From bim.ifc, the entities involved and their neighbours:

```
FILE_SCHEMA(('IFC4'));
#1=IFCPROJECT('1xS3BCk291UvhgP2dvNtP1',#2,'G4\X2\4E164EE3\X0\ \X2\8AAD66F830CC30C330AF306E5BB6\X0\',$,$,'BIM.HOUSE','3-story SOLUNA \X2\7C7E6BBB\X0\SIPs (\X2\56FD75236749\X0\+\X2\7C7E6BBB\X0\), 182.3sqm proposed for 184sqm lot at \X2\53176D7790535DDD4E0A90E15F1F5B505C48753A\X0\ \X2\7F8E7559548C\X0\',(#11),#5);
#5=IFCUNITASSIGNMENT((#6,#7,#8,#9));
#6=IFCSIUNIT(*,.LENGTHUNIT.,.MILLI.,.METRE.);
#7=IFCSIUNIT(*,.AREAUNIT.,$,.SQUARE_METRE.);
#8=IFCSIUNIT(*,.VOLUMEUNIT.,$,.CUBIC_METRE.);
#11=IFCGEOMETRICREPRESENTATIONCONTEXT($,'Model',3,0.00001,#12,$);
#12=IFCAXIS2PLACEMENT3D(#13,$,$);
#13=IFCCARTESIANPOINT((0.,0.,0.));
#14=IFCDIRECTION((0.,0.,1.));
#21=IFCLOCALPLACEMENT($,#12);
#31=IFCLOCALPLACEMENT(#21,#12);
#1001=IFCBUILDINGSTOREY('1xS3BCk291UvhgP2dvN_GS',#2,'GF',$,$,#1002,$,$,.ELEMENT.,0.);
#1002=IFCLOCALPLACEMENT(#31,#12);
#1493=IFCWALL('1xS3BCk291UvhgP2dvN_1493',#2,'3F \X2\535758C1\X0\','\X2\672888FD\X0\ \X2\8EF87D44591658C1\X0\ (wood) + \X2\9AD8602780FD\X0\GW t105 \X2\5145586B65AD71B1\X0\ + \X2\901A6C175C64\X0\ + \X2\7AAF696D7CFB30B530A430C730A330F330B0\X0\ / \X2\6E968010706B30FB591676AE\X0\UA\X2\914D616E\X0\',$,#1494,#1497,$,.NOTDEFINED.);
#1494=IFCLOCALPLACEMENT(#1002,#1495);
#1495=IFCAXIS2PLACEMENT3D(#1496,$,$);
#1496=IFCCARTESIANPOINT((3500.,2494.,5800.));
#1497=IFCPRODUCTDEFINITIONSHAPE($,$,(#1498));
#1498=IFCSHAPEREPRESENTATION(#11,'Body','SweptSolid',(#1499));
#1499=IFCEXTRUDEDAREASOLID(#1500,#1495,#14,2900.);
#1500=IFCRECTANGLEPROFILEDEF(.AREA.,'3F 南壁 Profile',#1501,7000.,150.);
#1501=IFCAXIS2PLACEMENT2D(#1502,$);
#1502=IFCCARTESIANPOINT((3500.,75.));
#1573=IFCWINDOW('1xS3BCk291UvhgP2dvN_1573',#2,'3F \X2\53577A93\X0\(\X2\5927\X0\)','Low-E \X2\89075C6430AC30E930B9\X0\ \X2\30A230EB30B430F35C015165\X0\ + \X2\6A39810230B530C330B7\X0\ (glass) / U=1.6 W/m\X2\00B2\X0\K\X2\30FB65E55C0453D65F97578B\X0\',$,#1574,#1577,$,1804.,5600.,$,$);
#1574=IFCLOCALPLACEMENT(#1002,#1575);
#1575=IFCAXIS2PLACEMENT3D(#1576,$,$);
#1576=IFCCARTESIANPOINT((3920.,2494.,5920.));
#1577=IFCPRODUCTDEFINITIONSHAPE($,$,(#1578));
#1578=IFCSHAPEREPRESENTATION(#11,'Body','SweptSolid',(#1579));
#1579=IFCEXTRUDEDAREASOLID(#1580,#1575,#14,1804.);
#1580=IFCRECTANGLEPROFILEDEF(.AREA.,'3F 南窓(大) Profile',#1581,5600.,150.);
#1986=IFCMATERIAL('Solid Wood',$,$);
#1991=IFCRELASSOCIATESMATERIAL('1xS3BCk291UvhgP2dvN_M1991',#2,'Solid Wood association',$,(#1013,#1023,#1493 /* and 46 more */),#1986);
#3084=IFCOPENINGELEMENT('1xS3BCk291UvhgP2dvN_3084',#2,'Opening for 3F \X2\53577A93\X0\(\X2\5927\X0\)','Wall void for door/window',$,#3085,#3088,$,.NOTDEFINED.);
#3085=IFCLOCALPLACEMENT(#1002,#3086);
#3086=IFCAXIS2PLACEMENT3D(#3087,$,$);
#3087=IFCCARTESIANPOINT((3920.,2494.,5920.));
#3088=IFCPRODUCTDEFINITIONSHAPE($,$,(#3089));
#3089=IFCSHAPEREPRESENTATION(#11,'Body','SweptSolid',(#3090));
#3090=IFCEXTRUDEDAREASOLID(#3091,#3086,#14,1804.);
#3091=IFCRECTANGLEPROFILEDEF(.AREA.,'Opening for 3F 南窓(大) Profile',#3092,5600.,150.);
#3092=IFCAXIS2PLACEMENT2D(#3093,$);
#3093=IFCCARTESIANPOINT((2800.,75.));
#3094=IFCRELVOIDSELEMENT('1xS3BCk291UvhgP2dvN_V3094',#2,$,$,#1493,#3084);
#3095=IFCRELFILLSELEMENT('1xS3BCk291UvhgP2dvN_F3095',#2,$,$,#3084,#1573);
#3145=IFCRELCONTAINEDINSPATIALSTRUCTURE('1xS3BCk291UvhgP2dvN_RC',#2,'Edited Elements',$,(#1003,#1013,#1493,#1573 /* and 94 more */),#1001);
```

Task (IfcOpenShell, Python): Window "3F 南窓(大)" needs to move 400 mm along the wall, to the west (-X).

```python
import ifcopenshell
import ifcopenshell.api.geometry
import ifcopenshell.util.placement

model = ifcopenshell.open("bim.ifc")

window = model.by_id(1573)
opening = window.FillsVoids[0].RelatingOpeningElement
wall = opening.VoidsElements[0].RelatingBuildingElement

wall_matrix = ifcopenshell.util.placement.get_local_placement(wall.ObjectPlacement)
shift = wall_matrix[:3, 0] * -400.0
before = ifcopenshell.util.placement.get_local_placement(window.ObjectPlacement)[:3, 3].copy()

# The window is not placed relative to its opening, so move both.
for product in (opening, window):
    matrix = ifcopenshell.util.placement.get_local_placement(product.ObjectPlacement)
    matrix[:3, 3] += shift
    ifcopenshell.api.geometry.edit_object_placement(model, product=product, matrix=matrix, is_si=False)

after = ifcopenshell.util.placement.get_local_placement(window.ObjectPlacement)[:3, 3]
print("window moved by", (after - before).round(3) + 0.0)

model.write("bim_v2.ifc")
```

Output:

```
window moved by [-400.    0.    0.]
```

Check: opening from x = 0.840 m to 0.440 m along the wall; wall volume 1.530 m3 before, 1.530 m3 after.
